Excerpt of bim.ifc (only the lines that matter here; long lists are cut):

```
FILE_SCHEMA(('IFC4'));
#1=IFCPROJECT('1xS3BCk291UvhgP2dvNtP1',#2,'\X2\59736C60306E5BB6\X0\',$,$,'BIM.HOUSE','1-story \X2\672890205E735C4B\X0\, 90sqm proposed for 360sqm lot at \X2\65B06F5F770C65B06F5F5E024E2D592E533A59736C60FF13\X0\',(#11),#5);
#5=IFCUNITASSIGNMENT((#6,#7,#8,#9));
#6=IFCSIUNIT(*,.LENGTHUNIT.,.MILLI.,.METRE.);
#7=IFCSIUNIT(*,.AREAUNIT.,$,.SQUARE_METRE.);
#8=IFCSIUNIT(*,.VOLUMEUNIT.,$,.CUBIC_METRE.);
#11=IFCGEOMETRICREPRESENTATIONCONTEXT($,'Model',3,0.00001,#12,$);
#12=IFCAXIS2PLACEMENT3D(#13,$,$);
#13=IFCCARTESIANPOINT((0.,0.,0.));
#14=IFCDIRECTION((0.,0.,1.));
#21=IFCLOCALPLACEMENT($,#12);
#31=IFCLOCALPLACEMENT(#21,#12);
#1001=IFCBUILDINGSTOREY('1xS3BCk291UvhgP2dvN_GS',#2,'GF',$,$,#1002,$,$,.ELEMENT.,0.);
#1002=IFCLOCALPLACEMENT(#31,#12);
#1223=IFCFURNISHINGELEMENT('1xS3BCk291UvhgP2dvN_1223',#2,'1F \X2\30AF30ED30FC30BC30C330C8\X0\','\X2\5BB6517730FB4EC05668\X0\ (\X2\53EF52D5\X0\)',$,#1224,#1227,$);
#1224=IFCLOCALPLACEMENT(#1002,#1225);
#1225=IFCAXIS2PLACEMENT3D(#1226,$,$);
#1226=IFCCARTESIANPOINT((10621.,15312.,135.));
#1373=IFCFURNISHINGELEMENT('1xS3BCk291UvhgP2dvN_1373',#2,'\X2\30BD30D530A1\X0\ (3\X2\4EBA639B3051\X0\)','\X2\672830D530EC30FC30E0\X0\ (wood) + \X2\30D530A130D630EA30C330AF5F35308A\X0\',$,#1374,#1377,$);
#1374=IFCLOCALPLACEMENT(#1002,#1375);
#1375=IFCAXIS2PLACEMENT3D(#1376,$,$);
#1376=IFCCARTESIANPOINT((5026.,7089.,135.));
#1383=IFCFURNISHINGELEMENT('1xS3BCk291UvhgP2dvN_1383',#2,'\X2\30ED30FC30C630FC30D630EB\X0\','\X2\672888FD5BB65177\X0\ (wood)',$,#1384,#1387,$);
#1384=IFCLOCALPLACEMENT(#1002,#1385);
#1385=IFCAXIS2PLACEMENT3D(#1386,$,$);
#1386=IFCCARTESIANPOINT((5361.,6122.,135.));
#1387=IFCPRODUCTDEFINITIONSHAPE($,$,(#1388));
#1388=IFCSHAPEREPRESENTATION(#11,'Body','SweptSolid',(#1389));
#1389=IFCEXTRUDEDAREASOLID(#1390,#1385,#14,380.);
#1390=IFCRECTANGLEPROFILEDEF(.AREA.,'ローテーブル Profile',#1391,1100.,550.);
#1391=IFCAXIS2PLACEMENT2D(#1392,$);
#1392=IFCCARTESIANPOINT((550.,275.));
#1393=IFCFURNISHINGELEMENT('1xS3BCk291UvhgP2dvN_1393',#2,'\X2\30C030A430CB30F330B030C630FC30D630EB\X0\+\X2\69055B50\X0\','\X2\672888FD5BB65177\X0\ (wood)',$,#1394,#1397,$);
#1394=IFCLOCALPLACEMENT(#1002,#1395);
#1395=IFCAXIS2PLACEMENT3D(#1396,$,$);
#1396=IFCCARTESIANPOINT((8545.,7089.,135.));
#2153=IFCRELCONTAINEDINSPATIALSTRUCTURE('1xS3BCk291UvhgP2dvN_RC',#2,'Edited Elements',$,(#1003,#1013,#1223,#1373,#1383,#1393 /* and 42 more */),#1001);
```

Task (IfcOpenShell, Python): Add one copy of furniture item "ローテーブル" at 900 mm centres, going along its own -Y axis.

```python
import ifcopenshell
import ifcopenshell.api.geometry
import ifcopenshell.api.root
import ifcopenshell.util.element
import ifcopenshell.util.placement
import ifcopenshell.util.unit

model = ifcopenshell.open("bim.ifc")
unit_scale = ifcopenshell.util.unit.calculate_unit_scale(model)


def reuse_history(source, copy):
    """copy_class also copies each property set's owner history, people and application; keep the originals."""
    for rel in copy.IsDefinedBy:
        if rel.is_a("IfcRelDefinesByProperties") and (history := rel.RelatingPropertyDefinition.OwnerHistory):
            rel.RelatingPropertyDefinition.OwnerHistory = source.OwnerHistory
            ifcopenshell.util.element.remove_deep2(model, history)


source = model.by_id(1383)
base = ifcopenshell.util.placement.get_local_placement(source.ObjectPlacement)
step = -base[:3, 1] * 0.9 / unit_scale

for i in range(1, 2):
    copy = ifcopenshell.api.root.copy_class(model, product=source)
    copy.Representation = ifcopenshell.util.element.copy_deep(
        model, source.Representation, exclude=["IfcGeometricRepresentationContext", "IfcRepresentationMap"]
    )
    reuse_history(source, copy)
    matrix = base.copy()
    matrix[:3, 3] += i * step
    print("added at", matrix[:3, 3].round(3) + 0.0)
    ifcopenshell.api.geometry.edit_object_placement(model, product=copy, matrix=matrix, is_si=False)

model.write("bim_edited.ifc")
```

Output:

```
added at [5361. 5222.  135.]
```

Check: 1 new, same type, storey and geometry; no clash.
